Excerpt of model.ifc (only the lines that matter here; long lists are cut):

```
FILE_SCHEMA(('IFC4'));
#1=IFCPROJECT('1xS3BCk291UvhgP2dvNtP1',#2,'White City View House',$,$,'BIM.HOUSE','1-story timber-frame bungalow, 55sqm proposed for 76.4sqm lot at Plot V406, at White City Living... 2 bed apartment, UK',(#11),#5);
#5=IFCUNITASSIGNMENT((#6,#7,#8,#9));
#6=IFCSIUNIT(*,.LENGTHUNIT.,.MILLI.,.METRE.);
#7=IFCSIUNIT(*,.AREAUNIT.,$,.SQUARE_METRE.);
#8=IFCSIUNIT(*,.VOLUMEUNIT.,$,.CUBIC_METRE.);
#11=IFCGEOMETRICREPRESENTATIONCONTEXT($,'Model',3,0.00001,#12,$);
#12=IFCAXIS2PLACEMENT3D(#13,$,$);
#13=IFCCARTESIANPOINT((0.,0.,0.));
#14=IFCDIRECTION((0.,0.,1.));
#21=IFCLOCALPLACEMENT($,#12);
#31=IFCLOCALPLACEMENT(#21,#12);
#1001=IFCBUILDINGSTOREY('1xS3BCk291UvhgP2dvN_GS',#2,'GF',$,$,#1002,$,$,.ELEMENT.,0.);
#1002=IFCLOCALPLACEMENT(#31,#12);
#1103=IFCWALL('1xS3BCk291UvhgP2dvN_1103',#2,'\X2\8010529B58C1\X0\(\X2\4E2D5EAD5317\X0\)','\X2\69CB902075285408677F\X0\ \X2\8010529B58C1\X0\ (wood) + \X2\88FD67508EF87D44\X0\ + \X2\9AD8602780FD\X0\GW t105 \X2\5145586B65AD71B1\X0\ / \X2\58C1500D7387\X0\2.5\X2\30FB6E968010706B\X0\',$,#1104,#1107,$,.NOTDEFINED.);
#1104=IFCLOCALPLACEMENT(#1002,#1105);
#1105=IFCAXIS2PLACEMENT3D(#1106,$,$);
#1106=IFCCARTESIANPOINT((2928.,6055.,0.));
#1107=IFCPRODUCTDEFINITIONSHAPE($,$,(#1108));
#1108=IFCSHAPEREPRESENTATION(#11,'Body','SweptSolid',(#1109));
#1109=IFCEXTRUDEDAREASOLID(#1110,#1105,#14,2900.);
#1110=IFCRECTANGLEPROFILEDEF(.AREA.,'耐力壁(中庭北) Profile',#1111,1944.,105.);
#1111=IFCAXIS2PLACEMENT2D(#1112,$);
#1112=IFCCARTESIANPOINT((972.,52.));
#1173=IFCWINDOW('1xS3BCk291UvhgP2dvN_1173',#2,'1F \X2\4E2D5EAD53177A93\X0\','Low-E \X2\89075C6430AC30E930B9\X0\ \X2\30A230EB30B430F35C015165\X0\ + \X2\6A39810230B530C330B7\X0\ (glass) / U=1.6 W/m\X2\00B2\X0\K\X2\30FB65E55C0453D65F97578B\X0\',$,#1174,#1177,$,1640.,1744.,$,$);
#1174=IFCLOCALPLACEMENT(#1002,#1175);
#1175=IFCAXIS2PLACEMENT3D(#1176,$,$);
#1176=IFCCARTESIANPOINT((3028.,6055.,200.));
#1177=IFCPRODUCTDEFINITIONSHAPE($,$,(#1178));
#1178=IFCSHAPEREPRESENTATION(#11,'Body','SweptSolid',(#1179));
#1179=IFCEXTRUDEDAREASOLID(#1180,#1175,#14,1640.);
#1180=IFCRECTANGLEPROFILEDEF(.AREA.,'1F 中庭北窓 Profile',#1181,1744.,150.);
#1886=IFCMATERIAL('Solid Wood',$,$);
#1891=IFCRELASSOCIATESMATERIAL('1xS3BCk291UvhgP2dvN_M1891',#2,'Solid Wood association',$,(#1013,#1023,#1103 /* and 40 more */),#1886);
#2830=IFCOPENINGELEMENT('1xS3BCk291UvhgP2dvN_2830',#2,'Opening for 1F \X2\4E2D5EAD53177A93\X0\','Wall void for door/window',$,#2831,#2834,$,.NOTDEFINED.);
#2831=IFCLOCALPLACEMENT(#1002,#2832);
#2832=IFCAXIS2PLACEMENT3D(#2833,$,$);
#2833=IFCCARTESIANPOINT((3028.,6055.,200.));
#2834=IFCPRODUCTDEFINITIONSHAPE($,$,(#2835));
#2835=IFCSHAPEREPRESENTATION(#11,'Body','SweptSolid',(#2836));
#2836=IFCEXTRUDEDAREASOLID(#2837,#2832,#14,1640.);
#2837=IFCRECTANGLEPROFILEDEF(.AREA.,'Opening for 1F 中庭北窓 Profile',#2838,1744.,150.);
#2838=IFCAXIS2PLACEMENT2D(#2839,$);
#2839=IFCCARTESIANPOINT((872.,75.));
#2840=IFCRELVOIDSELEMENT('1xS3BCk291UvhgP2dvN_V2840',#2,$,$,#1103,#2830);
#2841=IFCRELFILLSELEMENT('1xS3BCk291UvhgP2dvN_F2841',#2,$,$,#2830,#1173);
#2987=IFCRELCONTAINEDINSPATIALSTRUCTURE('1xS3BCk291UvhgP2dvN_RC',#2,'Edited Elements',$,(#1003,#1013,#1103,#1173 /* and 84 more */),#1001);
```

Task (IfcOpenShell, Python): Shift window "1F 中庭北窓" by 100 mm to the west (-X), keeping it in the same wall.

```python
import ifcopenshell
import ifcopenshell.api.geometry
import ifcopenshell.util.placement
import ifcopenshell.util.unit

model = ifcopenshell.open("model.ifc")
unit_scale = ifcopenshell.util.unit.calculate_unit_scale(model)

window = model.by_guid("1xS3BCk291UvhgP2dvN_1173")
opening = window.FillsVoids[0].RelatingOpeningElement
wall = opening.VoidsElements[0].RelatingBuildingElement

wall_matrix = ifcopenshell.util.placement.get_local_placement(wall.ObjectPlacement)
shift = wall_matrix[:3, 0] * -0.1 / unit_scale
before = ifcopenshell.util.placement.get_local_placement(window.ObjectPlacement)[:3, 3].copy()

# The window is not placed relative to its opening, so move both.
for product in (opening, window):
    matrix = ifcopenshell.util.placement.get_local_placement(product.ObjectPlacement)
    matrix[:3, 3] += shift
    ifcopenshell.api.geometry.edit_object_placement(model, product=product, matrix=matrix, is_si=False)

after = ifcopenshell.util.placement.get_local_placement(window.ObjectPlacement)[:3, 3]
print("window moved by", (after - before).round(3) + 0.0)

model.write("model_updated.ifc")
```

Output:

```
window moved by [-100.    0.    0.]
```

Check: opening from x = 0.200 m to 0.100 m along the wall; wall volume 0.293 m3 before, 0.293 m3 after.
